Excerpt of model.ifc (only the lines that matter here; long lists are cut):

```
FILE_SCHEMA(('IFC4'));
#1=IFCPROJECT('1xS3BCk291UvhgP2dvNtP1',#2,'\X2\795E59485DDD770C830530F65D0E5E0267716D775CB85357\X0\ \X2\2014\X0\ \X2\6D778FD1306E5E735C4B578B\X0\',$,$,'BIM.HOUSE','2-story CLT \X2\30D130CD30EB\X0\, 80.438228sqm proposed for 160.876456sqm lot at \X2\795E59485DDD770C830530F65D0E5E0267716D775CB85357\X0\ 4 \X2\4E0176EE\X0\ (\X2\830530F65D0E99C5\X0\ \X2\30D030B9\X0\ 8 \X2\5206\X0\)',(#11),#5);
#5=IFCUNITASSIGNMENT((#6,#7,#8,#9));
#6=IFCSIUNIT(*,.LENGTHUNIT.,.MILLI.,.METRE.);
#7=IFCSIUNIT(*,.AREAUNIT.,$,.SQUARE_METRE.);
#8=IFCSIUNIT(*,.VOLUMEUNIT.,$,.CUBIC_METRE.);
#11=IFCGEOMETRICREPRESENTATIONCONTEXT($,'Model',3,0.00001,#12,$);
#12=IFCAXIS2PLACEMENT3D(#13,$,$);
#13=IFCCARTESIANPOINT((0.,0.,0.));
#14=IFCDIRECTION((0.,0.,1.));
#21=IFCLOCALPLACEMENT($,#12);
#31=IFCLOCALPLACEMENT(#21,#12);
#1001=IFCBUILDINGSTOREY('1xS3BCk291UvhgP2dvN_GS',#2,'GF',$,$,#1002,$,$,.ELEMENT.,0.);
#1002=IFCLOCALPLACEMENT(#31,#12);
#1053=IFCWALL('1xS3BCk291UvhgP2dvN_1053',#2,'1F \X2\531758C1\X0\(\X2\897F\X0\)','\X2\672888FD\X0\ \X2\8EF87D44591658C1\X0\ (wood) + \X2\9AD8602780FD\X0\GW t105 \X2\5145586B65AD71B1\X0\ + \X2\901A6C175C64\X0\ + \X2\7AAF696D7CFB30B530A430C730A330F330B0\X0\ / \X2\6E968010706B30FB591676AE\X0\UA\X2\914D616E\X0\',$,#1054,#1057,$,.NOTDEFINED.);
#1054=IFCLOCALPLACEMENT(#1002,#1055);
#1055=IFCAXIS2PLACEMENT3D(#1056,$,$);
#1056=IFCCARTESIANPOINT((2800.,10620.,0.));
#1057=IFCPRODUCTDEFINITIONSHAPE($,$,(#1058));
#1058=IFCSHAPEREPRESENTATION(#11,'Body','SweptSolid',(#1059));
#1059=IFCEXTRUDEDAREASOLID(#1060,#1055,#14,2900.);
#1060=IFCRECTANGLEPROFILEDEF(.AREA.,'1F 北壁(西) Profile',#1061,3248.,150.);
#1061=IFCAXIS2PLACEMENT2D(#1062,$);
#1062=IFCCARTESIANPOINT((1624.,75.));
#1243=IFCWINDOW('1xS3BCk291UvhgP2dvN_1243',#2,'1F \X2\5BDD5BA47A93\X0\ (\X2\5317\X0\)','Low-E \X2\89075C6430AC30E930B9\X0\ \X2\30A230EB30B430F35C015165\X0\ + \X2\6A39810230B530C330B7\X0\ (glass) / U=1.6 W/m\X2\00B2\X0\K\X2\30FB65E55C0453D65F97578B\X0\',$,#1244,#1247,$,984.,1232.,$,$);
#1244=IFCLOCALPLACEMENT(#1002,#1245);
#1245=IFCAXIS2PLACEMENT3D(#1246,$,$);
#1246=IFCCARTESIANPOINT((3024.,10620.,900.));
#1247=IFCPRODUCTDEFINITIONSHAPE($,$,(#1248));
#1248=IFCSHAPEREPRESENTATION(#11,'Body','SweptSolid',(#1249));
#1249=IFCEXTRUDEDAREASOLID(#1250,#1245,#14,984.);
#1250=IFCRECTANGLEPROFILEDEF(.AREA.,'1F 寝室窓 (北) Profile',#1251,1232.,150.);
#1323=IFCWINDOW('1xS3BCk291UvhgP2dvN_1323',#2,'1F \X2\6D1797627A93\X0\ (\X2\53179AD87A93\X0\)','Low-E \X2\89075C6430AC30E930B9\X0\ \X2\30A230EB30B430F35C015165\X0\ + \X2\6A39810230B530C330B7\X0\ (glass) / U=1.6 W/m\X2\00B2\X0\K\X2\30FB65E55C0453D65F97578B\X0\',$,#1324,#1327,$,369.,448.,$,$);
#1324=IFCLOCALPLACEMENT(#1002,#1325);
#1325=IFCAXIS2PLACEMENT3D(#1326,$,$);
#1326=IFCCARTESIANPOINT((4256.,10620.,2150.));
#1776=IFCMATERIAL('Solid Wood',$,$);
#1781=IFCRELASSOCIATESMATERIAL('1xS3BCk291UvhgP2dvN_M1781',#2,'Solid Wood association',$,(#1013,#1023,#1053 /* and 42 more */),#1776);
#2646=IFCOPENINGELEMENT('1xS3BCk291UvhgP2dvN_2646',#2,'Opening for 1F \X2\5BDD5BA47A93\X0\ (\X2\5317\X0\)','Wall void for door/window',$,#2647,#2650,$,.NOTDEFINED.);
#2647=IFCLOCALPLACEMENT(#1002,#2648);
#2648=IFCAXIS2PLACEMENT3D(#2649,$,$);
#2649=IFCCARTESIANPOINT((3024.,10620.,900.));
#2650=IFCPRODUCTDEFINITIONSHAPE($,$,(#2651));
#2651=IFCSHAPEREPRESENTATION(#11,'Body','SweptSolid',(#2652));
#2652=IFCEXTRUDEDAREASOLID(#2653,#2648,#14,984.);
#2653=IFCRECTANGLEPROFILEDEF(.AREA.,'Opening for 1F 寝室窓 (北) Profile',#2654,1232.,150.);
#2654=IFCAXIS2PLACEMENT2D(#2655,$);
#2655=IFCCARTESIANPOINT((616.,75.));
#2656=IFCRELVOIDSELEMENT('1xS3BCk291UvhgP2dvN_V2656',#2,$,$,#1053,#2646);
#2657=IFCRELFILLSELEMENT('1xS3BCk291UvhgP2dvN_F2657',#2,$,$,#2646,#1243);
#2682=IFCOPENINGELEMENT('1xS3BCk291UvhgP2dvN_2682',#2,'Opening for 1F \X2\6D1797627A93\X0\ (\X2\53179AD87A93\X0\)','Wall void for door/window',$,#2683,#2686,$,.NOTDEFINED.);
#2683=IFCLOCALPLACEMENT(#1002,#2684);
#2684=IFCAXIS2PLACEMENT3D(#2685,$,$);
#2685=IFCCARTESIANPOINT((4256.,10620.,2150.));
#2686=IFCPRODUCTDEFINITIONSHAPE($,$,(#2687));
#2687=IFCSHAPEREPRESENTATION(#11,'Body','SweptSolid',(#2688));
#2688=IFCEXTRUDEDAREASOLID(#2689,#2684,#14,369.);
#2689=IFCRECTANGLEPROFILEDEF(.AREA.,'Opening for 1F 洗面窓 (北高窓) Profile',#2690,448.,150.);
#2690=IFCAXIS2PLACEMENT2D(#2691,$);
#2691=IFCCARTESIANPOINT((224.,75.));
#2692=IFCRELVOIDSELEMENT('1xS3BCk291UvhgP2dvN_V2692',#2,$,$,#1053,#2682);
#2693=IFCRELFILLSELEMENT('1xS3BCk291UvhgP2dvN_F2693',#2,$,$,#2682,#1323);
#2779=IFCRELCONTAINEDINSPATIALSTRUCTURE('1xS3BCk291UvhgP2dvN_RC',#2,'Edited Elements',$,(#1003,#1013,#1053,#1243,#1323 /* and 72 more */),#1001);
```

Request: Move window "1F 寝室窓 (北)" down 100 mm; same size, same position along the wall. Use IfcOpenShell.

```python
import numpy as np
import ifcopenshell
import ifcopenshell.api.geometry
import ifcopenshell.util.placement
import ifcopenshell.util.unit

model = ifcopenshell.open("model.ifc")
unit_scale = ifcopenshell.util.unit.calculate_unit_scale(model)

window = model.by_guid("1xS3BCk291UvhgP2dvN_1243")
opening = window.FillsVoids[0].RelatingOpeningElement
dz = -100.0

shift = np.array([0.0, 0.0, dz])
# The window is not placed relative to its opening, so move both.
for product in (opening, window):
    matrix = ifcopenshell.util.placement.get_local_placement(product.ObjectPlacement)
    matrix[:3, 3] += shift
    ifcopenshell.api.geometry.edit_object_placement(model, product=product, matrix=matrix, is_si=False)

print(f"moved by {dz * unit_scale:+.3f} m")

model.write("model_rev.ifc")
```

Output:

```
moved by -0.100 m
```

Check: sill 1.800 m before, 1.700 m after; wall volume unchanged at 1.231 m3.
